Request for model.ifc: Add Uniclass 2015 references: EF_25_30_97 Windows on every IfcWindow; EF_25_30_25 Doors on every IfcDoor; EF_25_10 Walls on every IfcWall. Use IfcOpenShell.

First a look at what the model holds.

```python
import ifcopenshell

model = ifcopenshell.open("model.ifc")
print(model.schema)
print("classifications:", [c.Name for c in model.by_type("IfcClassification")])
for ifc_class in ("IfcDoor", "IfcRoof", "IfcStair", "IfcWall", "IfcWindow"):
    print(ifc_class, len(model.by_type(ifc_class)))
```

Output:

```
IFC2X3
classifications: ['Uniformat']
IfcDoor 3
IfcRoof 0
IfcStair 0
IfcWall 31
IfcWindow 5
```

```python
import ifcopenshell
import ifcopenshell.api.classification

model = ifcopenshell.open("model.ifc")

# IFC2X3 requires Source and Edition and has no link from the project to the system.
system = model.create_entity("IfcClassification", Source="NBS", Edition="2015", Name="Uniclass 2015")

codes = {
    "IfcWindow": ("EF_25_30_97", "Windows"),
    "IfcDoor": ("EF_25_30_25", "Doors"),
    "IfcWall": ("EF_25_10", "Walls"),
}
for ifc_class, (code, name) in codes.items():
    products = model.by_type(ifc_class)
    ifcopenshell.api.classification.add_reference(
        model, products=products, classification=system, identification=code, name=name
    )
    print(code, len(products))

model.write("model_rev.ifc")
```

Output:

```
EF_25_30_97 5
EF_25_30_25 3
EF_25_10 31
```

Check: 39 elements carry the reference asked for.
